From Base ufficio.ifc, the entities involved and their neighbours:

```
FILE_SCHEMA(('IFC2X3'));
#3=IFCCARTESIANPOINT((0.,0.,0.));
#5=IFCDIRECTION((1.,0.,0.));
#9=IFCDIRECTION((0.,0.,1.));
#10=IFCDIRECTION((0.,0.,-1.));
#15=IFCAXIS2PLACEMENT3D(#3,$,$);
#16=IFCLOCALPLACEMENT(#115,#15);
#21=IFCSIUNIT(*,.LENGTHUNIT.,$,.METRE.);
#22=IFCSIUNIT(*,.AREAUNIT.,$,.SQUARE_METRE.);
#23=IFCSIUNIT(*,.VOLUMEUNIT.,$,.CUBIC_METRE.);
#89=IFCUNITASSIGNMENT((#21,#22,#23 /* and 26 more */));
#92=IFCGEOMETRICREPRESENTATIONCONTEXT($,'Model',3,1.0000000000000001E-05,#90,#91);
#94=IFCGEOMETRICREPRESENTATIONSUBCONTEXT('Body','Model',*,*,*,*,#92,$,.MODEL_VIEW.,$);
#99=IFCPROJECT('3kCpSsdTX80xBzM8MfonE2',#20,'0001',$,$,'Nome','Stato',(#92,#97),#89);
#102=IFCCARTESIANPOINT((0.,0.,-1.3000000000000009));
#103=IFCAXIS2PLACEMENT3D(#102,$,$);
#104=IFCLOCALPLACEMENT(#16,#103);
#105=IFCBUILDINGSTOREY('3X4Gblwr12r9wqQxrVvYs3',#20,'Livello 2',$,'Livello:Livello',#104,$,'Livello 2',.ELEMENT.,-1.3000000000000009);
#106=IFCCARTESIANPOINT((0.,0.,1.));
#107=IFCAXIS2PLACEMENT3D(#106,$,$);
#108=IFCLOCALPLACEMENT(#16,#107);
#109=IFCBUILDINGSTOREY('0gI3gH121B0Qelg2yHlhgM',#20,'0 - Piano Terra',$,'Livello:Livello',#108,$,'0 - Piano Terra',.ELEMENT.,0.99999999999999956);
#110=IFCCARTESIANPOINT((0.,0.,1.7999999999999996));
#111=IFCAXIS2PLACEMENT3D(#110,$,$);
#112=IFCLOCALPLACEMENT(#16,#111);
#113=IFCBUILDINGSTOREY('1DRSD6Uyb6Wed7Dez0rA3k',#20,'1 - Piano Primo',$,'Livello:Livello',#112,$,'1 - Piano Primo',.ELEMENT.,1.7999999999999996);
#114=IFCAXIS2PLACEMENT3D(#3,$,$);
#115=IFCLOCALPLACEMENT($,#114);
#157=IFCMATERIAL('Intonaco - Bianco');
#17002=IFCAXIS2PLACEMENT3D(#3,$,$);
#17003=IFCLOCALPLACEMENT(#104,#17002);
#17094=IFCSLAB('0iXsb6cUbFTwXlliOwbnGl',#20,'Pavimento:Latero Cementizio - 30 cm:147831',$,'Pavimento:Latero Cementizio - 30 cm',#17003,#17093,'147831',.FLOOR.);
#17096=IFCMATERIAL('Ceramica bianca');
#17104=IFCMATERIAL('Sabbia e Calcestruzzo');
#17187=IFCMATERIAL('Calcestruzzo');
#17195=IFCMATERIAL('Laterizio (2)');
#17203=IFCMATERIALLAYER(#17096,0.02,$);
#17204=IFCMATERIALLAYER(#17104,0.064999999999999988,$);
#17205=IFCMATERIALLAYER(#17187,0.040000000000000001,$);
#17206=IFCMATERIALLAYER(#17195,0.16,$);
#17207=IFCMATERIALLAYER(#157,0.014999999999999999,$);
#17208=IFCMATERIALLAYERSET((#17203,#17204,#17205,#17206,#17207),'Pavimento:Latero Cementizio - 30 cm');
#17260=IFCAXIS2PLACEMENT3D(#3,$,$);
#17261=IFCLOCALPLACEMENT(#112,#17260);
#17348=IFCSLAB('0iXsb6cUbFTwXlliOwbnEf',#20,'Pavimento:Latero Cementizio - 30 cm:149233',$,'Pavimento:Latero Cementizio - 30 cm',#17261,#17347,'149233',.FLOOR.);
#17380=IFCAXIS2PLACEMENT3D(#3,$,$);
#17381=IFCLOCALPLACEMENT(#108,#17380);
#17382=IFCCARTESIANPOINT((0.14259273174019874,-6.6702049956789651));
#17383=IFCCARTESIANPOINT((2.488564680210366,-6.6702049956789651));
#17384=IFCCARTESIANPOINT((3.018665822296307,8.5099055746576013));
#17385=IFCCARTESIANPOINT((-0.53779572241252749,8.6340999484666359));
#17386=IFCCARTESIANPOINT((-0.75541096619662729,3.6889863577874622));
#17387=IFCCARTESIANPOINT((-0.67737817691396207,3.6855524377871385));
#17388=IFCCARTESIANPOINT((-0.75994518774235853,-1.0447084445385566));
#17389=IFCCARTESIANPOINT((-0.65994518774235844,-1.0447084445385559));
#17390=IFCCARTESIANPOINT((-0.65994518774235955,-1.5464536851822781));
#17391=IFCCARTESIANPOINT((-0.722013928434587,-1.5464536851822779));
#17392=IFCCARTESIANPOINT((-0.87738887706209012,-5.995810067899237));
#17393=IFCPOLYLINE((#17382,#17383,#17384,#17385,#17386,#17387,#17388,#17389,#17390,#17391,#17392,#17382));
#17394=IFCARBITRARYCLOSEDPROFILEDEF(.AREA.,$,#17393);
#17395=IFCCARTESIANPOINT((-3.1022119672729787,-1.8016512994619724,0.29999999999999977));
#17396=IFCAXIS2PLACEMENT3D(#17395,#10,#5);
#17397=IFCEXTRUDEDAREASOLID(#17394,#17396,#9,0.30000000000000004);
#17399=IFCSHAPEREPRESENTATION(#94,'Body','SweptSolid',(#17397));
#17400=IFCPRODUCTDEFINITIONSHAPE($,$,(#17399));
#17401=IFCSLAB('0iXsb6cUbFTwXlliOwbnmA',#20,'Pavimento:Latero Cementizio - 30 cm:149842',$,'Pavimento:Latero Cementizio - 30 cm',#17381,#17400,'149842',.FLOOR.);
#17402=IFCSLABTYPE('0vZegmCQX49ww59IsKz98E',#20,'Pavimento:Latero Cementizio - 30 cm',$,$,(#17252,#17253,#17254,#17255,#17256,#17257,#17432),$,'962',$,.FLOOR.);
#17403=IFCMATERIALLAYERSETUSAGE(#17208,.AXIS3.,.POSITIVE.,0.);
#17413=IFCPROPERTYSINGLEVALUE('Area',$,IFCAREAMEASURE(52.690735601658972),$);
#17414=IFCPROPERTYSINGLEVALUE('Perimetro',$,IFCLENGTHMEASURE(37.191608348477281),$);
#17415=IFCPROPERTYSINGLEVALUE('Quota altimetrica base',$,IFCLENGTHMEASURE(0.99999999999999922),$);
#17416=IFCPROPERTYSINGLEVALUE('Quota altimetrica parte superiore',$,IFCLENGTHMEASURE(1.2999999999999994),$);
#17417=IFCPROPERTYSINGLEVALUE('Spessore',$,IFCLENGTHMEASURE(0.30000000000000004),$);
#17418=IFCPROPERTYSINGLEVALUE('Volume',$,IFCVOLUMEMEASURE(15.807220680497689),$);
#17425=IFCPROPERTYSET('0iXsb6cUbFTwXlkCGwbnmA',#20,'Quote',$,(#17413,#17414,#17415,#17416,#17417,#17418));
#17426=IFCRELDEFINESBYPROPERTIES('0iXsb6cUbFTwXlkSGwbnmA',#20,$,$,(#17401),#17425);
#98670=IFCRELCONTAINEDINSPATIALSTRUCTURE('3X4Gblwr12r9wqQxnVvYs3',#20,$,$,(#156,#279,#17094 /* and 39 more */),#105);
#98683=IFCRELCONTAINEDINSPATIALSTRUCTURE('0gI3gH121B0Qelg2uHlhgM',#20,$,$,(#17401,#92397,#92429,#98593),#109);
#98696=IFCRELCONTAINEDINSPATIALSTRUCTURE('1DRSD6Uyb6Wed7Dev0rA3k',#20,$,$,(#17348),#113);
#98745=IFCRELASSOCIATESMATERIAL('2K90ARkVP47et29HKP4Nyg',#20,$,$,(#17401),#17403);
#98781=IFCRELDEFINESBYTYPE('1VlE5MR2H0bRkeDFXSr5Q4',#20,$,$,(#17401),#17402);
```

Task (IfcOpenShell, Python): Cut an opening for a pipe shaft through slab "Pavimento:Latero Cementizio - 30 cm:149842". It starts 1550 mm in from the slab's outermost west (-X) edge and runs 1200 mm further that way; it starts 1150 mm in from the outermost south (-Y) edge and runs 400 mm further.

```python
import numpy as np
import ifcopenshell
import ifcopenshell.api.feature
import ifcopenshell.api.geometry
import ifcopenshell.api.pset
import ifcopenshell.api.root
import ifcopenshell.geom
import ifcopenshell.util.element
import ifcopenshell.util.placement
import ifcopenshell.util.representation
import ifcopenshell.util.shape
import ifcopenshell.util.unit

model = ifcopenshell.open("Base ufficio.ifc")
unit_scale = ifcopenshell.util.unit.calculate_unit_scale(model)
area_scale = ifcopenshell.util.unit.calculate_unit_scale(model, "AREAUNIT")
volume_scale = ifcopenshell.util.unit.calculate_unit_scale(model, "VOLUMEUNIT")
settings = ifcopenshell.geom.settings()


def volume(element):
    """Net volume in cubic metres, openings subtracted."""
    shape = ifcopenshell.geom.create_shape(settings, element)
    return ifcopenshell.util.shape.get_volume(shape.geometry)


slab = model.by_guid("0iXsb6cUbFTwXlliOwbnmA")
before = volume(slab)

# Extent in the slab's own axes, in metres. The edges named are its -X and -Y sides.
slab_shape = ifcopenshell.geom.create_shape(settings, slab)
vertices = ifcopenshell.util.shape.get_vertices(slab_shape.geometry)
x_min, y_min, bottom = vertices.min(axis=0)
top = vertices[:, 2].max()

opening = ifcopenshell.api.root.create_entity(model, ifc_class="IfcOpeningElement", name="Pipe shaft opening")
context = ifcopenshell.util.representation.get_context(model, "Model", "Body", "MODEL_VIEW")
width, depth = 1.2, 0.4
outline = [(0.0, 0.0), (width, 0.0), (width, depth), (0.0, depth), (0.0, 0.0)]
# Overshoot both faces by 50 mm so the cut is clean.
shape = ifcopenshell.api.geometry.add_slab_representation(
    model, context=context, depth=top - bottom + 0.1, polyline=outline
)
ifcopenshell.api.geometry.assign_representation(model, product=opening, representation=shape)

matrix = ifcopenshell.util.placement.get_local_placement(slab.ObjectPlacement)
matrix[:, 3] = matrix @ np.append(np.array([x_min + 1.55, y_min + 1.15, bottom - 0.05]) / unit_scale, 1.0)
ifcopenshell.api.geometry.edit_object_placement(model, product=opening, matrix=matrix, is_si=False)
ifcopenshell.api.feature.add_feature(model, feature=opening, element=slab)

after = volume(slab)

# Update the slab's stored quantities.
pset = model.by_id(ifcopenshell.util.element.get_pset(slab, "Quote", should_inherit=False)["id"])
ifcopenshell.api.pset.edit_pset(model, pset=pset, properties={
    "Area": model.create_entity("IfcAreaMeasure", after / (top - bottom) / area_scale),
    "Volume": model.create_entity("IfcVolumeMeasure", after / volume_scale),
})

print(f"slab volume {before:.3f} -> {after:.3f} m3")

model.write("Base ufficio_edited.ifc")
```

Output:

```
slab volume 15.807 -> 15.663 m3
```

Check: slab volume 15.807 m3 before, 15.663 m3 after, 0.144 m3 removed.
